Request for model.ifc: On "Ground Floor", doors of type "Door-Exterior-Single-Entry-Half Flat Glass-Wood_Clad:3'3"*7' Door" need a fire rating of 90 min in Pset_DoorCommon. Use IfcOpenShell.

First a look at what the model holds.

```python
import ifcopenshell
import ifcopenshell.util.element

model = ifcopenshell.open("model.ifc")
print(model.schema)
storey = next(s for s in model.by_type("IfcBuildingStorey") if s.Name == "Ground Floor")
doors = [e for e in ifcopenshell.util.element.get_decomposition(storey) if e.is_a("IfcDoor")]
seen = {}
for e in doors:
    element_type = ifcopenshell.util.element.get_type(e)
    key = (element_type.Name if element_type != e and element_type else None, ifcopenshell.util.element.get_pset(e, "Pset_DoorCommon", "FireRating"))
    seen[key] = seen.get(key, 0) + 1
for (name, value), count in sorted(seen.items(), key=str):
    print(count, "x", name, "|", value)
```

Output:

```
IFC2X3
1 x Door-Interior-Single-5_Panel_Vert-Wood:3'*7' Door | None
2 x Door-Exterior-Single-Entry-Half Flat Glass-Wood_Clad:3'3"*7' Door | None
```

```python
import ifcopenshell
import ifcopenshell.api.pset
import ifcopenshell.util.element

model = ifcopenshell.open("model.ifc")

storey = next(s for s in model.by_type("IfcBuildingStorey") if s.Name == "Ground Floor")
doors = [e for e in ifcopenshell.util.element.get_decomposition(storey) if e.is_a("IfcDoor")]

count = 0
for e in doors:
    element_type = ifcopenshell.util.element.get_type(e)
    if element_type in (None, e) or element_type.Name != 'Door-Exterior-Single-Entry-Half Flat Glass-Wood_Clad:3\'3"*7\' Door':
        continue
    # add_pset returns the element's existing set when there is one.
    pset = ifcopenshell.api.pset.add_pset(model, product=e, name="Pset_DoorCommon")
    ifcopenshell.api.pset.edit_pset(model, pset=pset, properties={"FireRating": "90 min"})
    count += 1

print(count, "doors updated")

model.write("model_edited.ifc")
```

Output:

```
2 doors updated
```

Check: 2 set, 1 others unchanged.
